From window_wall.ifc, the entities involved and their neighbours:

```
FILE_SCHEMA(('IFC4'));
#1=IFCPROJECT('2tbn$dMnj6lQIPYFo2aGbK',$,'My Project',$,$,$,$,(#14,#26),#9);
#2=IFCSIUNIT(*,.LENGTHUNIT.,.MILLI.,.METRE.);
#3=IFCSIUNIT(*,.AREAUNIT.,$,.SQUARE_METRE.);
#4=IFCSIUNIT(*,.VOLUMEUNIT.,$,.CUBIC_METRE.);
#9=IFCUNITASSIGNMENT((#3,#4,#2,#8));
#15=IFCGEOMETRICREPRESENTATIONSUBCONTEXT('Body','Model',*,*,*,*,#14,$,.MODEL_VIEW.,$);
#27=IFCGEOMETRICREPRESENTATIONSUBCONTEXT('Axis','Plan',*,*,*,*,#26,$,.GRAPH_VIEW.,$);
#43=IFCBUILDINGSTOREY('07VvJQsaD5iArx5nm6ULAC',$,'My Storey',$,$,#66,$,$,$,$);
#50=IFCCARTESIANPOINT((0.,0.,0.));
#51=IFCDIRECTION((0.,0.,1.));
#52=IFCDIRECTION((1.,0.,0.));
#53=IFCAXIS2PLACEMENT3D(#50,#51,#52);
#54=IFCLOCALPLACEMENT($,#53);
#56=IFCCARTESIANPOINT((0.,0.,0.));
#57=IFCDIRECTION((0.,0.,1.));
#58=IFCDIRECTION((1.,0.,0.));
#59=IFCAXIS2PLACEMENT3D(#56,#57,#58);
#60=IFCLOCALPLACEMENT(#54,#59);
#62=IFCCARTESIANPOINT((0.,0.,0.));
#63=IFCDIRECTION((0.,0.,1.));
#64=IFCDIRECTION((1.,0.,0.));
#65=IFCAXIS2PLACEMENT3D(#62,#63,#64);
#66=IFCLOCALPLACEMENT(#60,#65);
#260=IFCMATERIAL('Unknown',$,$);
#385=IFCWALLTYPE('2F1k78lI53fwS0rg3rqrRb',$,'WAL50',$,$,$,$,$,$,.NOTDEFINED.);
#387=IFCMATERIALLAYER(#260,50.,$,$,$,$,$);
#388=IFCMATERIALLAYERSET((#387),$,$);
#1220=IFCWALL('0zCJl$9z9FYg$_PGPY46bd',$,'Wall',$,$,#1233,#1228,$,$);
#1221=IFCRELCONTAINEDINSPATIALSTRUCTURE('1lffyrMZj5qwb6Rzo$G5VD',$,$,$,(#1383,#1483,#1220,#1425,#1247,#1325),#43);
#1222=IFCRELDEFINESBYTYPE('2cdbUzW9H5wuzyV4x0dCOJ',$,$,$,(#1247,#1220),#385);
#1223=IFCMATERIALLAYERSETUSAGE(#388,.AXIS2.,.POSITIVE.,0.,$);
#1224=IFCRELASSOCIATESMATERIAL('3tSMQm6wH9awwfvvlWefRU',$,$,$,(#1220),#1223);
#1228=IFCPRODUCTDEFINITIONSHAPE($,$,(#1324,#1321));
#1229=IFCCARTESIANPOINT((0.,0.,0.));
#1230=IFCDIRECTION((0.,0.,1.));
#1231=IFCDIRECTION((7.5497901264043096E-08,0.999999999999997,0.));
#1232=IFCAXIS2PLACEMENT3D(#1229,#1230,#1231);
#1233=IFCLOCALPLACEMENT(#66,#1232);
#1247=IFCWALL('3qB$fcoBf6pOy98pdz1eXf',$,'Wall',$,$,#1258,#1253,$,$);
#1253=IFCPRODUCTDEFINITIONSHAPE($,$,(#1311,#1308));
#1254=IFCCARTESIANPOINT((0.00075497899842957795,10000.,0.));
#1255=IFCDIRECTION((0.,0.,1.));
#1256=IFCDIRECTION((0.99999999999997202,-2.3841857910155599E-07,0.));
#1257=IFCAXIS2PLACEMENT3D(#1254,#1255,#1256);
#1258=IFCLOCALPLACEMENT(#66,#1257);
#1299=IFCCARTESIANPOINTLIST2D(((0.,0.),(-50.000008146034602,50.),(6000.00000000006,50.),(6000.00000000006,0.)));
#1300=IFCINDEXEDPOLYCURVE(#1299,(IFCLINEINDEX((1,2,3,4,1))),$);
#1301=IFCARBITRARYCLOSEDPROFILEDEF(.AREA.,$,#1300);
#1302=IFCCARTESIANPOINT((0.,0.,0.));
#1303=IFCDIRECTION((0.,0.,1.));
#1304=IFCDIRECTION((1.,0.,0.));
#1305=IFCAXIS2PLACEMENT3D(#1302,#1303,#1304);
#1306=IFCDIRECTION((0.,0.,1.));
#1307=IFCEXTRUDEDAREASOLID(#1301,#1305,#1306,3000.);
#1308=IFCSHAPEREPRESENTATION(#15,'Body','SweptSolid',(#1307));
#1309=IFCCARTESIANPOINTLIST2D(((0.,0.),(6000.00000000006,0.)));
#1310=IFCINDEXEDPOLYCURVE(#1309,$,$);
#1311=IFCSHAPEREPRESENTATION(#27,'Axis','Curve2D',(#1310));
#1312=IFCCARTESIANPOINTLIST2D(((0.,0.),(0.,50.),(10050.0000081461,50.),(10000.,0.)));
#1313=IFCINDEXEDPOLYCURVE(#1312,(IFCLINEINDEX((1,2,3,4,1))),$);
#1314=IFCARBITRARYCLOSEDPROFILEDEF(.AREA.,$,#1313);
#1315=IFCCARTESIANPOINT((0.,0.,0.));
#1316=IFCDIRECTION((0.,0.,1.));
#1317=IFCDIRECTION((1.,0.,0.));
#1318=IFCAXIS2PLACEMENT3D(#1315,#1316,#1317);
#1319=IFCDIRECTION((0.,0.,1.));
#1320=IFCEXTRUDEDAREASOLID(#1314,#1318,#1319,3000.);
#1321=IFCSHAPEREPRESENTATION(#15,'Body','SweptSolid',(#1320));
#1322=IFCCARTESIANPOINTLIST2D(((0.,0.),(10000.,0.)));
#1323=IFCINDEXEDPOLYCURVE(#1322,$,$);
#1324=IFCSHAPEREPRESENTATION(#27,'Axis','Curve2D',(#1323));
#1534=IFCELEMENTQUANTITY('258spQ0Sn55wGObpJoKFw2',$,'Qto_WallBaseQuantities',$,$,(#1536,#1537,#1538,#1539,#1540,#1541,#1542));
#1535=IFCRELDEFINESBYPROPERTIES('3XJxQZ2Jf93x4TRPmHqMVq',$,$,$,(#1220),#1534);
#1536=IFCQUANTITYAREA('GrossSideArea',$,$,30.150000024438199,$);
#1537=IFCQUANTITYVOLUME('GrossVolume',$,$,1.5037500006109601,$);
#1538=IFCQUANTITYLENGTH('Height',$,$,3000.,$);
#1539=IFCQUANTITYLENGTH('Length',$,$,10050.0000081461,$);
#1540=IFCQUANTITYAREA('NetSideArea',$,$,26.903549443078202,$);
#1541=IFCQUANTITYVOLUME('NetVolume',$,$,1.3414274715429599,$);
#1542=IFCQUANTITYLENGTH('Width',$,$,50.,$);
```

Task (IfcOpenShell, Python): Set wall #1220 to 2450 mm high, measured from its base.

```python
import ifcopenshell
import ifcopenshell.api.pset
import ifcopenshell.geom
import ifcopenshell.util.element
import ifcopenshell.util.representation
import ifcopenshell.util.shape
import ifcopenshell.util.unit

model = ifcopenshell.open("window_wall.ifc")
unit_scale = ifcopenshell.util.unit.calculate_unit_scale(model)
area_scale = ifcopenshell.util.unit.calculate_unit_scale(model, "AREAUNIT")
volume_scale = ifcopenshell.util.unit.calculate_unit_scale(model, "VOLUMEUNIT")
settings = ifcopenshell.geom.settings()


def volume(element):
    """Net volume in cubic metres, openings subtracted."""
    shape = ifcopenshell.geom.create_shape(settings, element)
    return ifcopenshell.util.shape.get_volume(shape.geometry)


wall = model.by_id(1220)
before = volume(wall)

body = ifcopenshell.util.representation.get_representation(wall, "Model", "Body")
solid = body.Items[0]
old_height = solid.Depth
solid.Depth = 2.45 / unit_scale
after = volume(wall)
thickness = 0.05  # wall thickness in metres

# Update the stored height, areas and volumes.
qto = model.by_id(ifcopenshell.util.element.get_pset(wall, "Qto_WallBaseQuantities", should_inherit=False)["id"])
ifcopenshell.api.pset.edit_qto(model, qto=qto, properties={
    "GrossSideArea": ifcopenshell.util.element.get_pset(wall, "Qto_WallBaseQuantities", "GrossSideArea") * solid.Depth / old_height,
    "GrossVolume": ifcopenshell.util.element.get_pset(wall, "Qto_WallBaseQuantities", "GrossVolume") * solid.Depth / old_height,
    "Height": solid.Depth,
    "NetSideArea": after / thickness / area_scale,
    "NetVolume": after / volume_scale,
})

print(f"height {old_height:g} -> {solid.Depth:g}, volume {before:.3f} -> {after:.3f} m3")

model.write("window_wall-out.ifc")
```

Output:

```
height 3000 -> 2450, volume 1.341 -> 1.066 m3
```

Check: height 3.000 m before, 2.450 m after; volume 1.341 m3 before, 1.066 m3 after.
